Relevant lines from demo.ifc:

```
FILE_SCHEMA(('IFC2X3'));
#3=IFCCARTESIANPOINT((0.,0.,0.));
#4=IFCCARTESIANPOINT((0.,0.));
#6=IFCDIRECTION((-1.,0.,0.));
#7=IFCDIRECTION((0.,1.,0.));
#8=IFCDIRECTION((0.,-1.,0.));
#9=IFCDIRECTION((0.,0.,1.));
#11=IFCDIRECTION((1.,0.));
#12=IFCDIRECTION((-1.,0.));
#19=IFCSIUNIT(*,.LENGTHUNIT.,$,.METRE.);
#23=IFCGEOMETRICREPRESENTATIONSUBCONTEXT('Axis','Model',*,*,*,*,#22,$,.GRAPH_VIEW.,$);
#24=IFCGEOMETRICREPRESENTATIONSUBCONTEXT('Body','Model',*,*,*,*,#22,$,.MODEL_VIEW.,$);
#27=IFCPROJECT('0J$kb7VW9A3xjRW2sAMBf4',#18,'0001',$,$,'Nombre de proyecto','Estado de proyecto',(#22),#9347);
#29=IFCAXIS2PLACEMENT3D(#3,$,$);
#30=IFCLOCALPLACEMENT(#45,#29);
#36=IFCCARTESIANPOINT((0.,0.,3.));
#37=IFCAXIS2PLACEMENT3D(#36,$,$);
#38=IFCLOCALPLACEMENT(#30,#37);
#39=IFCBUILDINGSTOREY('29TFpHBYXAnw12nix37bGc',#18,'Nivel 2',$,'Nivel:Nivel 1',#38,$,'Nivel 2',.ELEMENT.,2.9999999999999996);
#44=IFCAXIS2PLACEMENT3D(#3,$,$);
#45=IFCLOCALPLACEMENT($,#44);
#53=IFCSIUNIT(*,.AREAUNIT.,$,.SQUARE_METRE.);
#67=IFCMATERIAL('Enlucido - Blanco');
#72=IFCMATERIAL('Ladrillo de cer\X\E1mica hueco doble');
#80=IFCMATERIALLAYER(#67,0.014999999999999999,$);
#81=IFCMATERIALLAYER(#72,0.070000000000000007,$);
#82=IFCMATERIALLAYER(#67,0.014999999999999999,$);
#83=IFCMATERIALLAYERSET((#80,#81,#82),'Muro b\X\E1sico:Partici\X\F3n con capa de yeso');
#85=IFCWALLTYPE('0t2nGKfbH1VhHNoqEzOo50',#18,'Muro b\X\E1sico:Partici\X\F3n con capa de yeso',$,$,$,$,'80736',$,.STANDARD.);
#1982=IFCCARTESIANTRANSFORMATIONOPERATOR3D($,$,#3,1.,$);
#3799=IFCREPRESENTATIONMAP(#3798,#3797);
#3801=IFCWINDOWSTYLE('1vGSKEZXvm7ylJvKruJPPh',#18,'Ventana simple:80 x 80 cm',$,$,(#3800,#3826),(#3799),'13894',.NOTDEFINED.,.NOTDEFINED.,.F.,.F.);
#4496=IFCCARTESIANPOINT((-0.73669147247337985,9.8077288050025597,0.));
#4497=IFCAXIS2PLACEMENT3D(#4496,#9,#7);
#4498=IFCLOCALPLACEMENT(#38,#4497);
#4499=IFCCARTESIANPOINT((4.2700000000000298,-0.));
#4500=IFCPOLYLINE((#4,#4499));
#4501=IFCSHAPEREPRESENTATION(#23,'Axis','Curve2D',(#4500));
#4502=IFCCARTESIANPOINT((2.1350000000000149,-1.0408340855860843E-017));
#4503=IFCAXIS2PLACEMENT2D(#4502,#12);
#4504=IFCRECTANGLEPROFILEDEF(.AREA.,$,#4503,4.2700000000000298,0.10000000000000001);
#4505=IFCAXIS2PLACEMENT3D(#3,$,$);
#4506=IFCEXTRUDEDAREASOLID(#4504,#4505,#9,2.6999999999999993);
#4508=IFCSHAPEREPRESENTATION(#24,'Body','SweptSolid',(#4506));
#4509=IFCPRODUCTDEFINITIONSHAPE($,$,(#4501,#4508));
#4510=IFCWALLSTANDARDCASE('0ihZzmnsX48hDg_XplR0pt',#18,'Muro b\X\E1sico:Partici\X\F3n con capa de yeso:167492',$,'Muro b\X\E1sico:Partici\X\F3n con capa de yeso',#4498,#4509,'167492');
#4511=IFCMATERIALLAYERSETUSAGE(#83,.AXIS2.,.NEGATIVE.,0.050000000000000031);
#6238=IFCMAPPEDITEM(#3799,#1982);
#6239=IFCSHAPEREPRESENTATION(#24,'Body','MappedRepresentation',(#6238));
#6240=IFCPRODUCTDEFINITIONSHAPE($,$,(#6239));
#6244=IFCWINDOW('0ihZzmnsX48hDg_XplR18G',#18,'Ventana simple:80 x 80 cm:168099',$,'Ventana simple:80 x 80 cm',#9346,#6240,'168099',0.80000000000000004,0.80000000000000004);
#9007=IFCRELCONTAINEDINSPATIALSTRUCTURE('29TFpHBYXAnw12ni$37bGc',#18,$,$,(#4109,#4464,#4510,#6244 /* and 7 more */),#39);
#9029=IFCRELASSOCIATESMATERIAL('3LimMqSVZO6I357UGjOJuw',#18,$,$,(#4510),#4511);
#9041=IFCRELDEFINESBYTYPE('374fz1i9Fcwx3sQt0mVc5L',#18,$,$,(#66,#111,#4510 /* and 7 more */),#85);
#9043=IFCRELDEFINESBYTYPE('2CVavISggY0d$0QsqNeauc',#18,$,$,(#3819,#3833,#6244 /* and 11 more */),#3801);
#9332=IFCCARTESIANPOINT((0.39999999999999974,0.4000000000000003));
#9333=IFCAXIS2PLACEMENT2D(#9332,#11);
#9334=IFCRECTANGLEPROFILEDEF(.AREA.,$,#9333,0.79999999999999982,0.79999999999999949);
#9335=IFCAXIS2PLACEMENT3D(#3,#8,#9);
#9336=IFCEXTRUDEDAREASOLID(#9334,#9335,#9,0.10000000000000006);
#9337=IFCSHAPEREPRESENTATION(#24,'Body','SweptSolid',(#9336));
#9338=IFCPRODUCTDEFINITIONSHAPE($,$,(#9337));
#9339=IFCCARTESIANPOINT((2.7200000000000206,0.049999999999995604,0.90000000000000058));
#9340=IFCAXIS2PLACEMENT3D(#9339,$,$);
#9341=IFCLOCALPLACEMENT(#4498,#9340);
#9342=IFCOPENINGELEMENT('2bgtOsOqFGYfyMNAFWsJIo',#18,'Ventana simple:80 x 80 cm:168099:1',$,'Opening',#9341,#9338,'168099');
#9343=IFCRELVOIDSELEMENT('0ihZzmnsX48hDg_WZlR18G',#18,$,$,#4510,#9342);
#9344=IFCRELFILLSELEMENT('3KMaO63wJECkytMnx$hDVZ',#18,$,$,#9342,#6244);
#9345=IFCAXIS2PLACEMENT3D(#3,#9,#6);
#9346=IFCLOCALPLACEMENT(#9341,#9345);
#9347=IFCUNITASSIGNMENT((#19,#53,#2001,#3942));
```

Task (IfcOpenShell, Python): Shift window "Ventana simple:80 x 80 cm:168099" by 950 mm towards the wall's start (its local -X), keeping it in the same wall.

```python
import ifcopenshell
import ifcopenshell.api.geometry
import ifcopenshell.util.placement

model = ifcopenshell.open("demo.ifc")

window = model.by_id(6244)
opening = window.FillsVoids[0].RelatingOpeningElement
wall = opening.VoidsElements[0].RelatingBuildingElement

wall_matrix = ifcopenshell.util.placement.get_local_placement(wall.ObjectPlacement)
shift = wall_matrix[:3, 0] * -0.95
before = ifcopenshell.util.placement.get_local_placement(window.ObjectPlacement)[:3, 3].copy()

# The window is placed relative to its opening, so it follows when the opening moves.
matrix = ifcopenshell.util.placement.get_local_placement(opening.ObjectPlacement)
matrix[:3, 3] += shift
ifcopenshell.api.geometry.edit_object_placement(
    model, product=opening, matrix=matrix, is_si=False, should_transform_children=True
)

after = ifcopenshell.util.placement.get_local_placement(window.ObjectPlacement)[:3, 3]
print("window moved by", (after - before).round(3) + 0.0)

model.write("demo-out.ifc")
```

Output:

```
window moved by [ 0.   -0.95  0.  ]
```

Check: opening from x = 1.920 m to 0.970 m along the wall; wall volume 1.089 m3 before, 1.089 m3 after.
